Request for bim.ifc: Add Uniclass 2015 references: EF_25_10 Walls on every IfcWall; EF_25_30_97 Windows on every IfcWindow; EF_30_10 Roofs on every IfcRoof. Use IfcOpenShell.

First a look at what the model holds.

```python
import ifcopenshell

model = ifcopenshell.open("bim.ifc")
print(model.schema)
print("classifications:", [c.Name for c in model.by_type("IfcClassification")])
for ifc_class in ("IfcDoor", "IfcRoof", "IfcStair", "IfcWall", "IfcWindow"):
    print(ifc_class, len(model.by_type(ifc_class)))
```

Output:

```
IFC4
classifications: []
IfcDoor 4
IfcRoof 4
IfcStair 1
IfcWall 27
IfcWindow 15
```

```python
import ifcopenshell
import ifcopenshell.api.classification

model = ifcopenshell.open("bim.ifc")

system = ifcopenshell.api.classification.add_classification(model, classification="Uniclass 2015")

codes = {
    "IfcWall": ("EF_25_10", "Walls"),
    "IfcWindow": ("EF_25_30_97", "Windows"),
    "IfcRoof": ("EF_30_10", "Roofs"),
}
for ifc_class, (code, name) in codes.items():
    products = model.by_type(ifc_class)
    ifcopenshell.api.classification.add_reference(
        model, products=products, classification=system, identification=code, name=name
    )
    print(code, len(products))

model.write("bim_rev.ifc")
```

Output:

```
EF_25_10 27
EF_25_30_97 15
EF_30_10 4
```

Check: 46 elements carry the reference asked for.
